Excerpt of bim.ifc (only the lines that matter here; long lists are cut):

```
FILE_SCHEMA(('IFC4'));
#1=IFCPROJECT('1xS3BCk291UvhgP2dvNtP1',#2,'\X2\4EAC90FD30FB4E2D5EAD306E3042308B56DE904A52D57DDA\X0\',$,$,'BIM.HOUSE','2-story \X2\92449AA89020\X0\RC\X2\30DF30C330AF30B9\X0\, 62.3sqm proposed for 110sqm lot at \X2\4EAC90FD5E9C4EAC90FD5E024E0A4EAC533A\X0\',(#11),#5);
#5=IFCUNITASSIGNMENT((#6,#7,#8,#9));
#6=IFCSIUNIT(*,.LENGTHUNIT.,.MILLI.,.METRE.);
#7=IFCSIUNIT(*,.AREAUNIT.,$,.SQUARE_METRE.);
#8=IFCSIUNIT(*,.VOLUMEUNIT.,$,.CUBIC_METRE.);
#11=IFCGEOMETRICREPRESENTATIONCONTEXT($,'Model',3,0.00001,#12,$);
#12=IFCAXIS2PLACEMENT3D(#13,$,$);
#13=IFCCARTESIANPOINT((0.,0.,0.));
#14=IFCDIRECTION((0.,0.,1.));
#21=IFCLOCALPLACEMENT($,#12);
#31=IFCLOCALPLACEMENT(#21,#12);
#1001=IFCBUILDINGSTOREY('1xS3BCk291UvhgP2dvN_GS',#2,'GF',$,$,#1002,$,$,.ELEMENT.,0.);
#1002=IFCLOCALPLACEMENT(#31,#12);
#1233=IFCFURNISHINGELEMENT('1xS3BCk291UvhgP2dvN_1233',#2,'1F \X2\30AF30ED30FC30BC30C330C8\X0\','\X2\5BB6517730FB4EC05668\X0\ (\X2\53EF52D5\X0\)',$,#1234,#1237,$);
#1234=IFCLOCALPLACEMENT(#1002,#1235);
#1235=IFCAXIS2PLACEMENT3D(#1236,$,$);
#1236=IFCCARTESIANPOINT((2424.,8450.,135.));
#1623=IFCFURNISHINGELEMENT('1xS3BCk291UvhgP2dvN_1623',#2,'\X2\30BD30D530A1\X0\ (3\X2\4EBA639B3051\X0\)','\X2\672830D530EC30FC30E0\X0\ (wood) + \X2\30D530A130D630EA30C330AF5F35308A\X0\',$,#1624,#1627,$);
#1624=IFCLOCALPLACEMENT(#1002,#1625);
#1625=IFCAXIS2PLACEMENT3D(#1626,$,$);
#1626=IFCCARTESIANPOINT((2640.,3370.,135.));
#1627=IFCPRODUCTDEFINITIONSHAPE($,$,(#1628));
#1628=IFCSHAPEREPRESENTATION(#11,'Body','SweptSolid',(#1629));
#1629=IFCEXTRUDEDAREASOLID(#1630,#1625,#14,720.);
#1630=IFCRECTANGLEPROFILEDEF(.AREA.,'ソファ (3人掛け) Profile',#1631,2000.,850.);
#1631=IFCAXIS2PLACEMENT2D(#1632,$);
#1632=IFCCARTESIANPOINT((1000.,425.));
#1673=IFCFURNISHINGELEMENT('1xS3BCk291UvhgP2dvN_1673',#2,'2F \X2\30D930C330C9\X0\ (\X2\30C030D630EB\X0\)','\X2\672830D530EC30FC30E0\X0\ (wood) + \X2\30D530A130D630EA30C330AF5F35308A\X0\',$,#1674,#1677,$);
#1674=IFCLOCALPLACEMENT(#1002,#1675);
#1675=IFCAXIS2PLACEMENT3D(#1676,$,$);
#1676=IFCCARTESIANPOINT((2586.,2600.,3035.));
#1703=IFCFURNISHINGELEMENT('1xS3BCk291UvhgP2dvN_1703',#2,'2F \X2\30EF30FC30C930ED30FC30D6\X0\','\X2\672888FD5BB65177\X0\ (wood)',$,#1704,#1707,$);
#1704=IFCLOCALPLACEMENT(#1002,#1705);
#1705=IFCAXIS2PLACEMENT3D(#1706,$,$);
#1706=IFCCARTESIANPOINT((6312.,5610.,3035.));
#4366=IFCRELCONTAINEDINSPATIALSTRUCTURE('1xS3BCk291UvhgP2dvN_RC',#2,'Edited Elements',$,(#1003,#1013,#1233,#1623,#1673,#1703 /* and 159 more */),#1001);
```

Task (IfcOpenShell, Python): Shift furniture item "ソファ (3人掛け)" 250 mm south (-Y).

```python
import ifcopenshell
import ifcopenshell.api.geometry
import ifcopenshell.util.placement
import ifcopenshell.util.unit

model = ifcopenshell.open("bim.ifc")
unit_scale = ifcopenshell.util.unit.calculate_unit_scale(model)

item = model.by_id(1623)
matrix = ifcopenshell.util.placement.get_local_placement(item.ObjectPlacement)
matrix[1, 3] -= 0.25 / unit_scale
ifcopenshell.api.geometry.edit_object_placement(model, product=item, matrix=matrix, is_si=False)

print(ifcopenshell.util.placement.get_local_placement(item.ObjectPlacement).round(3) + 0.0)

model.write("bim_edited.ifc")
```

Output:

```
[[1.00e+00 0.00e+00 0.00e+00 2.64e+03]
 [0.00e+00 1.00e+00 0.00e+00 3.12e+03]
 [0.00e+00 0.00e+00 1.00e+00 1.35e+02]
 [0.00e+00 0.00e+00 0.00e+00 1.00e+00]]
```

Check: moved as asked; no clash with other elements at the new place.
